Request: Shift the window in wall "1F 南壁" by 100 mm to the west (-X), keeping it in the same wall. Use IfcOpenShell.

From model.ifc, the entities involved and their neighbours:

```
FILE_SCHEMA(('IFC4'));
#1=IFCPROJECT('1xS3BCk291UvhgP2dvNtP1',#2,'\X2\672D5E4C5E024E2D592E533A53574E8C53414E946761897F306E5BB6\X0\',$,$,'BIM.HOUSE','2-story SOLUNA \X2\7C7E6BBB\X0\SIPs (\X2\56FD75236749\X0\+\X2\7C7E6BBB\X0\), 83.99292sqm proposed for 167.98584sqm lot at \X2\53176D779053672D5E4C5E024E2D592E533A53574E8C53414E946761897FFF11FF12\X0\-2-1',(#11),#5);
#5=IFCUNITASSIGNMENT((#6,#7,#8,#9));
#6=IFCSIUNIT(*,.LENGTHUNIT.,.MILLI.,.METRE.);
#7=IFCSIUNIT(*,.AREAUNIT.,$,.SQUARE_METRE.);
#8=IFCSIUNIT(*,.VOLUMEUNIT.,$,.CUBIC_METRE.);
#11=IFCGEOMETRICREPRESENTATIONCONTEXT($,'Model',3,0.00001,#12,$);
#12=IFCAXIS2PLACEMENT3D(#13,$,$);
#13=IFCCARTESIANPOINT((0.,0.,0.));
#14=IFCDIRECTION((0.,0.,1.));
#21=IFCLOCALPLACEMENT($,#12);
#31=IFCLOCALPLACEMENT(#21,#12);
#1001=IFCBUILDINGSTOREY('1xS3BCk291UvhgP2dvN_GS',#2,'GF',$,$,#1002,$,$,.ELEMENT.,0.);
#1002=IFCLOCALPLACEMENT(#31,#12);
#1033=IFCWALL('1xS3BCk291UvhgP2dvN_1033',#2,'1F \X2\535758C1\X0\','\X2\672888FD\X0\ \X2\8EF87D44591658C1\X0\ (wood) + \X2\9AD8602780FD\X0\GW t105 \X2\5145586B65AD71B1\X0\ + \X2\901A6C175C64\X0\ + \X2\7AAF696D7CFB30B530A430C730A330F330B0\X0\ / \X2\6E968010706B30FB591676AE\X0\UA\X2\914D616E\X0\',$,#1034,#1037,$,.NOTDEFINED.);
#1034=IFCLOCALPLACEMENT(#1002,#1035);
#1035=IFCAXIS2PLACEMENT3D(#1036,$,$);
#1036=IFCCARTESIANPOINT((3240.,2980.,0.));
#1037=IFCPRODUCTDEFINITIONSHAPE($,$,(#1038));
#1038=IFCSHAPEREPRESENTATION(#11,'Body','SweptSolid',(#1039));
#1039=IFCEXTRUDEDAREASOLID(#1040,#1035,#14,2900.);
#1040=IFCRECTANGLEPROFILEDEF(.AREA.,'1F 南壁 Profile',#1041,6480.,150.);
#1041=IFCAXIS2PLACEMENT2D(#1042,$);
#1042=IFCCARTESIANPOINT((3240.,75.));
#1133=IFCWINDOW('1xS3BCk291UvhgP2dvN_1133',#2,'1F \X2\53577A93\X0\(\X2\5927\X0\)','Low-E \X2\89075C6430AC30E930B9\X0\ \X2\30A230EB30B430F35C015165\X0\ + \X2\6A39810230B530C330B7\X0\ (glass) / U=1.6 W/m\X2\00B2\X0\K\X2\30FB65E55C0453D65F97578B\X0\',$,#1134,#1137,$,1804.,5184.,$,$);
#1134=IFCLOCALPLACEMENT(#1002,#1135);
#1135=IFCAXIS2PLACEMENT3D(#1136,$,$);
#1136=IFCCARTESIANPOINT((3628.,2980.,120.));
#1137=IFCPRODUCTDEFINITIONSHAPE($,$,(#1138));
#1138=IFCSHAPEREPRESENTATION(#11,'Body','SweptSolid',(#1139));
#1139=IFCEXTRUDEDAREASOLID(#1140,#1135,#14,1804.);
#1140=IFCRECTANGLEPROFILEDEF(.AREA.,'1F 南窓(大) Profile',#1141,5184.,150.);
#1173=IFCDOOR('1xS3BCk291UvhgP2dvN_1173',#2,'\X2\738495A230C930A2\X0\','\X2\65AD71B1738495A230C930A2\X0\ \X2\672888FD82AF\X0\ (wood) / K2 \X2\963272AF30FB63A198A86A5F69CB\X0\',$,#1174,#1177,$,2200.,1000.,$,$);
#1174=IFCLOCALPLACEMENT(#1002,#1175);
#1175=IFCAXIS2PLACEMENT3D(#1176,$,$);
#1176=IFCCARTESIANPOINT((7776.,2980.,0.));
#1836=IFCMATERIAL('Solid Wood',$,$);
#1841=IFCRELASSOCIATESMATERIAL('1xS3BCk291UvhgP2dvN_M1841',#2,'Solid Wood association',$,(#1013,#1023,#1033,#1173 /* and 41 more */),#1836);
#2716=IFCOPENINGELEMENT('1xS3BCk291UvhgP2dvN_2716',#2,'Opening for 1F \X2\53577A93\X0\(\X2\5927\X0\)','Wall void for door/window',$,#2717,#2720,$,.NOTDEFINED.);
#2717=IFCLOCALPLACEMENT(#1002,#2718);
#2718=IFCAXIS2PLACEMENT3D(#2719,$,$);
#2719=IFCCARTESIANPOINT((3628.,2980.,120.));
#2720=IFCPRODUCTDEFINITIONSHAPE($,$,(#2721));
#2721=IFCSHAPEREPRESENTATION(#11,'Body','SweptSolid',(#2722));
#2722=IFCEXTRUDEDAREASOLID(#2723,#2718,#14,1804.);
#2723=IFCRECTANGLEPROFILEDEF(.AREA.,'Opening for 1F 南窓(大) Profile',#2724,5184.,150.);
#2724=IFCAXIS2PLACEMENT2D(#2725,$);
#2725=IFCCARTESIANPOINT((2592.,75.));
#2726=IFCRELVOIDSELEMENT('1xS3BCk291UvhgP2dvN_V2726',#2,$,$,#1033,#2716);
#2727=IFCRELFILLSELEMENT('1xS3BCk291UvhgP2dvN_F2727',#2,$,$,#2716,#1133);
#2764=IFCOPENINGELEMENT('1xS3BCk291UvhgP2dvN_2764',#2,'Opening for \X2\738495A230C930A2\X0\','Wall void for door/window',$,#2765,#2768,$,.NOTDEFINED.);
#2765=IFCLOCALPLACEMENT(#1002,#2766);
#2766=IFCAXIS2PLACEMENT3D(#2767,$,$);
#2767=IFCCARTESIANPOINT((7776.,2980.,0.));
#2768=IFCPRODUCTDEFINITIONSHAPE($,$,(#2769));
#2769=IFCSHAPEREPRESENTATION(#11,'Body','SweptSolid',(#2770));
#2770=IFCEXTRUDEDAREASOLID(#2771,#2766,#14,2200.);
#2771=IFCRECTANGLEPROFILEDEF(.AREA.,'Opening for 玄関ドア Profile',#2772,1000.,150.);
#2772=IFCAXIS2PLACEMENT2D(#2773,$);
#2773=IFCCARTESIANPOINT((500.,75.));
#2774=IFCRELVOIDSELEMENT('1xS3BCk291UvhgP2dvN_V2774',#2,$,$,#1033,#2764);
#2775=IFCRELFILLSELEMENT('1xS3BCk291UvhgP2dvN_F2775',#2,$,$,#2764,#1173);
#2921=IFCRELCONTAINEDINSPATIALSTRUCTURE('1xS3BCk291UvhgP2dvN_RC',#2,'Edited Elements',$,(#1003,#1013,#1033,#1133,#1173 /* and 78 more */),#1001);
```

```python
import ifcopenshell
import ifcopenshell.api.geometry
import ifcopenshell.util.placement
import ifcopenshell.util.unit

model = ifcopenshell.open("model.ifc")
unit_scale = ifcopenshell.util.unit.calculate_unit_scale(model)

window = model.by_id(1133)
opening = window.FillsVoids[0].RelatingOpeningElement
wall = opening.VoidsElements[0].RelatingBuildingElement

wall_matrix = ifcopenshell.util.placement.get_local_placement(wall.ObjectPlacement)
shift = wall_matrix[:3, 0] * -0.1 / unit_scale
before = ifcopenshell.util.placement.get_local_placement(window.ObjectPlacement)[:3, 3].copy()

# The window is not placed relative to its opening, so move both.
for product in (opening, window):
    matrix = ifcopenshell.util.placement.get_local_placement(product.ObjectPlacement)
    matrix[:3, 3] += shift
    ifcopenshell.api.geometry.edit_object_placement(model, product=product, matrix=matrix, is_si=False)

after = ifcopenshell.util.placement.get_local_placement(window.ObjectPlacement)[:3, 3]
print("window moved by", (after - before).round(3) + 0.0)

model.write("model_updated.ifc")
```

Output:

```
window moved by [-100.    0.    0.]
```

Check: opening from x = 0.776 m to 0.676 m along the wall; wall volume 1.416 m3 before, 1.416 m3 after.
